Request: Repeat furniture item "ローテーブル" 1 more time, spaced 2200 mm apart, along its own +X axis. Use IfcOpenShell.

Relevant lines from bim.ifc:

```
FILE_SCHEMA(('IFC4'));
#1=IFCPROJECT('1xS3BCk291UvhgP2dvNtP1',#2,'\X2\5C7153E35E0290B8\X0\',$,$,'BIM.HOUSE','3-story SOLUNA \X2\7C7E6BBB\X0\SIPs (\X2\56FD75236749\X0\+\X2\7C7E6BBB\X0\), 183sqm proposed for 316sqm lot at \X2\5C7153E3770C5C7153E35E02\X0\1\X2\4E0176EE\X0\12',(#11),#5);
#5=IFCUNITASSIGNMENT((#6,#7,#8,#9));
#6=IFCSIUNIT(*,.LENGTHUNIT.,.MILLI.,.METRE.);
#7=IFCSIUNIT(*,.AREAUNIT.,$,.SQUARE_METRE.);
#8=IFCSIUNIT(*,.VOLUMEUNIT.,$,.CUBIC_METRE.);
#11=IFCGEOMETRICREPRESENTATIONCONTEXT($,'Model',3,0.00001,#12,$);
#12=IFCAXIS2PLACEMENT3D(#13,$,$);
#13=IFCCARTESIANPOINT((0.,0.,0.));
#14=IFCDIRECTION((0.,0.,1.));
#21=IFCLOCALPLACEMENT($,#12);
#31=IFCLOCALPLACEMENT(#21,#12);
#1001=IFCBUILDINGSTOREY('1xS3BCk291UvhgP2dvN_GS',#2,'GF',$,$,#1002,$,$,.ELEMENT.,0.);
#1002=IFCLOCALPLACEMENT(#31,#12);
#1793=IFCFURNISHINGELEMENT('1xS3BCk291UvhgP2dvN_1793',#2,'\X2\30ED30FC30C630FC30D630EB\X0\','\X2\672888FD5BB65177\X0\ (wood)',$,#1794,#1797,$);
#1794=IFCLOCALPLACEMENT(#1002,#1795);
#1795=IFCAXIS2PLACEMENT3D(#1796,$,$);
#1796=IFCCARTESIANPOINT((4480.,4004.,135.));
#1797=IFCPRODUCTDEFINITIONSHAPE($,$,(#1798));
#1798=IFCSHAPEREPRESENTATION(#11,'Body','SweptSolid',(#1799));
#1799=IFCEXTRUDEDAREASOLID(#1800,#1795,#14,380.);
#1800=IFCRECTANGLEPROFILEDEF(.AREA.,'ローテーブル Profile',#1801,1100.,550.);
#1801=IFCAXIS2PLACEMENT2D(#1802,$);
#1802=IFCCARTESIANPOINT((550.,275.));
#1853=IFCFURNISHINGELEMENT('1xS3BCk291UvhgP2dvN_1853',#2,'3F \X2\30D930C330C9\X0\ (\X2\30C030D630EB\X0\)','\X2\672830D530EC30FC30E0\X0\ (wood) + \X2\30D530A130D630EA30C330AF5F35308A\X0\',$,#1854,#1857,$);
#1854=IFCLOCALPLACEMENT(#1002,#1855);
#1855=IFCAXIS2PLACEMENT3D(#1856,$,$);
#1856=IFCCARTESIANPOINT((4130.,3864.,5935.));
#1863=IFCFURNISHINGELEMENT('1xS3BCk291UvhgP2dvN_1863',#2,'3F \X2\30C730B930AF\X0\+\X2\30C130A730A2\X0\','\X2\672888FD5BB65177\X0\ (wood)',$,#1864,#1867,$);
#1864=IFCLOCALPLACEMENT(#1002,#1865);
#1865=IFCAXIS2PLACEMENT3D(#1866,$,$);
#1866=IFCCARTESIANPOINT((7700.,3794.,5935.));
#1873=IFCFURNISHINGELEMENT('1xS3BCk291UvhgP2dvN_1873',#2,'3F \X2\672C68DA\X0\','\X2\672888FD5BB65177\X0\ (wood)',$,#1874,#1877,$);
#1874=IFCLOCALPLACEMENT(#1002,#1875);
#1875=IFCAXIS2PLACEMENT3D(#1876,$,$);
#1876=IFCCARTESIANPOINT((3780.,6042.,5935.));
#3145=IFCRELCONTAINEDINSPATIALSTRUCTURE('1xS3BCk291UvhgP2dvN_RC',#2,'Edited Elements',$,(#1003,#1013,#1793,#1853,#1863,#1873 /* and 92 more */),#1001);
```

```python
import ifcopenshell
import ifcopenshell.api.geometry
import ifcopenshell.api.root
import ifcopenshell.util.element
import ifcopenshell.util.placement

model = ifcopenshell.open("bim.ifc")


def reuse_history(source, copy):
    """copy_class also copies each property set's owner history, people and application; keep the originals."""
    for rel in copy.IsDefinedBy:
        if rel.is_a("IfcRelDefinesByProperties") and (history := rel.RelatingPropertyDefinition.OwnerHistory):
            rel.RelatingPropertyDefinition.OwnerHistory = source.OwnerHistory
            ifcopenshell.util.element.remove_deep2(model, history)


source = model.by_id(1793)
base = ifcopenshell.util.placement.get_local_placement(source.ObjectPlacement)
step = base[:3, 0] * 2200.0

for i in range(1, 2):
    copy = ifcopenshell.api.root.copy_class(model, product=source)
    copy.Representation = ifcopenshell.util.element.copy_deep(
        model, source.Representation, exclude=["IfcGeometricRepresentationContext", "IfcRepresentationMap"]
    )
    reuse_history(source, copy)
    matrix = base.copy()
    matrix[:3, 3] += i * step
    print("added at", matrix[:3, 3].round(3) + 0.0)
    ifcopenshell.api.geometry.edit_object_placement(model, product=copy, matrix=matrix, is_si=False)

model.write("bim_rev.ifc")
```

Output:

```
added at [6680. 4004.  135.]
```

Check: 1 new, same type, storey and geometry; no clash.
